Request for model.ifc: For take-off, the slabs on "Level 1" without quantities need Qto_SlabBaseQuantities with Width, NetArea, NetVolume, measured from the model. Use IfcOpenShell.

First a look at what the model holds.

```python
import ifcopenshell
import ifcopenshell.util.element
import ifcopenshell.util.unit

model = ifcopenshell.open("model.ifc")
print(model.schema)
for unit_type in ("LENGTHUNIT", "AREAUNIT", "VOLUMEUNIT"):
    print(unit_type, ifcopenshell.util.unit.calculate_unit_scale(model, unit_type))
storey = next(s for s in model.by_type("IfcBuildingStorey") if s.Name == "Level 1")
slabs = [e for e in ifcopenshell.util.element.get_decomposition(storey) if e.is_a("IfcSlab")]
for e in sorted(slabs, key=lambda e: e.id()):
    print(e.id(), e.is_a(), e.Name, list(ifcopenshell.util.element.get_psets(e, qtos_only=True)), sep=" | ")
```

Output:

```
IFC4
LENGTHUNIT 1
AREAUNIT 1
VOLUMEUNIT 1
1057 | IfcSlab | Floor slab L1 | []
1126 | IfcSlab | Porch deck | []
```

```python
import ifcopenshell
import ifcopenshell.api.pset
import ifcopenshell.geom
import ifcopenshell.util.element
import ifcopenshell.util.shape
import ifcopenshell.util.unit

model = ifcopenshell.open("model.ifc")
unit_scale = ifcopenshell.util.unit.calculate_unit_scale(model)
area_scale = ifcopenshell.util.unit.calculate_unit_scale(model, "AREAUNIT")
volume_scale = ifcopenshell.util.unit.calculate_unit_scale(model, "VOLUMEUNIT")
settings = ifcopenshell.geom.settings()

storey = next(s for s in model.by_type("IfcBuildingStorey") if s.Name == "Level 1")
slabs = [e for e in ifcopenshell.util.element.get_decomposition(storey) if e.is_a("IfcSlab")]

for e in sorted(slabs, key=lambda e: e.id()):
    if ifcopenshell.util.element.get_psets(e, qtos_only=True, should_inherit=False):
        continue
    # Geometry comes back in metres, in the element's own axes.
    shape = ifcopenshell.geom.create_shape(settings, e)
    values = {
        "Width": ifcopenshell.util.shape.get_z(shape.geometry) / unit_scale,
        "NetArea": ifcopenshell.util.shape.get_footprint_area(shape.geometry) / area_scale,
        "NetVolume": ifcopenshell.util.shape.get_volume(shape.geometry) / volume_scale,
    }
    qto = ifcopenshell.api.pset.add_qto(model, product=e, name="Qto_SlabBaseQuantities")
    ifcopenshell.api.pset.edit_qto(model, qto=qto, properties=values)
    print(e.id(), {k: round(v, 3) for k, v in values.items()})

model.write("model_rev.ifc")
```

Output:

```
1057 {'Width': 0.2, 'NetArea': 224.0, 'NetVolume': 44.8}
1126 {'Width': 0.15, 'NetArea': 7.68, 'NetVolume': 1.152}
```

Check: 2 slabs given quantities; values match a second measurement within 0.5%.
